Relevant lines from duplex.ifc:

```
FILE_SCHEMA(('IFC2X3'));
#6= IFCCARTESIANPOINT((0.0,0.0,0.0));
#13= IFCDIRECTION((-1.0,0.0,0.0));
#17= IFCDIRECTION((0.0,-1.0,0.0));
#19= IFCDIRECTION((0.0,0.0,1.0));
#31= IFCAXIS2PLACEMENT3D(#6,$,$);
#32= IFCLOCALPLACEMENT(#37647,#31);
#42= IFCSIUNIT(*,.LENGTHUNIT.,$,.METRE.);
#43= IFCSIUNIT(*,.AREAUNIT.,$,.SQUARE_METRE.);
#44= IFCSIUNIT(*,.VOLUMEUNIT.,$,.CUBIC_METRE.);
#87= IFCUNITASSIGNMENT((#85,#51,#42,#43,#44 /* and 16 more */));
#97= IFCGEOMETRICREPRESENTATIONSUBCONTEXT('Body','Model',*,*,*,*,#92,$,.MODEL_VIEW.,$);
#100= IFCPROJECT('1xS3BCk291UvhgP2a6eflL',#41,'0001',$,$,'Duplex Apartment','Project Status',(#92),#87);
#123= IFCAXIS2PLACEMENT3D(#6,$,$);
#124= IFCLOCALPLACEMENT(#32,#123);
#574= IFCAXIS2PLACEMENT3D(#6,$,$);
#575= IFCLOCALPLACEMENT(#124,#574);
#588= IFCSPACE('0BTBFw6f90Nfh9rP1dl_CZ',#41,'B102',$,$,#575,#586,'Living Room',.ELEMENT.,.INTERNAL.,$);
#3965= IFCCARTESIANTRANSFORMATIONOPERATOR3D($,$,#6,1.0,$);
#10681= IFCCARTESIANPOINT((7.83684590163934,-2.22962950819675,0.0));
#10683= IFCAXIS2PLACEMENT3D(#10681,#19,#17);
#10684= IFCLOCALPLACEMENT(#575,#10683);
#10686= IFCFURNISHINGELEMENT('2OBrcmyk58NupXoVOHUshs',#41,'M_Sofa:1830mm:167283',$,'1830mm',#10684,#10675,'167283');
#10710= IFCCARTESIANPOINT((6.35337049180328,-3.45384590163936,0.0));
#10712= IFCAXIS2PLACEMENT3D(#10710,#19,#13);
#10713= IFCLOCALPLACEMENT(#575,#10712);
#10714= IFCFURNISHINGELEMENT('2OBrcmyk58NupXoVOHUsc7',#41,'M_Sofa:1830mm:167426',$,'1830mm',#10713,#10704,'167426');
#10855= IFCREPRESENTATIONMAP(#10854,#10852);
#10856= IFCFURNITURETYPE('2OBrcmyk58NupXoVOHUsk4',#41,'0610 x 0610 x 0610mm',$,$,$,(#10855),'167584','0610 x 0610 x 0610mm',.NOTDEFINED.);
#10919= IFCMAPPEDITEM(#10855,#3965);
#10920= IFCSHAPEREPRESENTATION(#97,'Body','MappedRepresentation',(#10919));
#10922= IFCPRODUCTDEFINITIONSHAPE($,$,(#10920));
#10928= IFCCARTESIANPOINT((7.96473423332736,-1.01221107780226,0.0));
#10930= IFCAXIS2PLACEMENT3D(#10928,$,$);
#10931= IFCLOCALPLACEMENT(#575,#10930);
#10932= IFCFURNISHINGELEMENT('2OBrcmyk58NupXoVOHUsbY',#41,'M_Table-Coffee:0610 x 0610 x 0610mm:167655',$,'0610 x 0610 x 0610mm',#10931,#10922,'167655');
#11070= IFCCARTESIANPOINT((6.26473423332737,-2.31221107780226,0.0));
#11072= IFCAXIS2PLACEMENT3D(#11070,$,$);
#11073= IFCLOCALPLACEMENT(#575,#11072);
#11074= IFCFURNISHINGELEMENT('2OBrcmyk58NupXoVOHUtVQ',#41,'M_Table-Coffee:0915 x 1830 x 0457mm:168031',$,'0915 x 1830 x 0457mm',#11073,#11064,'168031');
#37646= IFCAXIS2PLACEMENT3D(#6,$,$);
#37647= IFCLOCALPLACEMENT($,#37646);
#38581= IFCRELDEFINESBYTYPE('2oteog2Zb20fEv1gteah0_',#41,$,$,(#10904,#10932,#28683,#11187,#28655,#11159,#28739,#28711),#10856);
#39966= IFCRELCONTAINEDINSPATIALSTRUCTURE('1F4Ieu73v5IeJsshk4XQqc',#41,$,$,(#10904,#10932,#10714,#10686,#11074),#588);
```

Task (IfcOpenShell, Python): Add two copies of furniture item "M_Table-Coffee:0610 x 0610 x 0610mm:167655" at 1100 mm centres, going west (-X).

```python
import numpy as np
import ifcopenshell
import ifcopenshell.api.geometry
import ifcopenshell.api.root
import ifcopenshell.util.element
import ifcopenshell.util.placement
import ifcopenshell.util.unit

model = ifcopenshell.open("duplex.ifc")
unit_scale = ifcopenshell.util.unit.calculate_unit_scale(model)


def reuse_history(source, copy):
    """copy_class also copies each property set's owner history, people and application; keep the originals."""
    for rel in copy.IsDefinedBy:
        if rel.is_a("IfcRelDefinesByProperties") and (history := rel.RelatingPropertyDefinition.OwnerHistory):
            rel.RelatingPropertyDefinition.OwnerHistory = source.OwnerHistory
            ifcopenshell.util.element.remove_deep2(model, history)


source = model.by_guid("2OBrcmyk58NupXoVOHUsbY")
base = ifcopenshell.util.placement.get_local_placement(source.ObjectPlacement)
step = np.array([-1.0, 0.0, 0.0]) * 1.1 / unit_scale

for i in range(1, 3):
    copy = ifcopenshell.api.root.copy_class(model, product=source)
    copy.Representation = ifcopenshell.util.element.copy_deep(
        model, source.Representation, exclude=["IfcGeometricRepresentationContext", "IfcRepresentationMap"]
    )
    copy.Name = "M_Table-Coffee:0610 x 0610 x 0610mm"
    copy.Tag = None
    reuse_history(source, copy)
    matrix = base.copy()
    matrix[:3, 3] += i * step
    print("added at", matrix[:3, 3].round(3) + 0.0)
    ifcopenshell.api.geometry.edit_object_placement(model, product=copy, matrix=matrix, is_si=False)

model.write("duplex_v2.ifc")
```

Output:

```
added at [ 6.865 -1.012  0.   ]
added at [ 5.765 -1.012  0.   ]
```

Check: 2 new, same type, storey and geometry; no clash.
